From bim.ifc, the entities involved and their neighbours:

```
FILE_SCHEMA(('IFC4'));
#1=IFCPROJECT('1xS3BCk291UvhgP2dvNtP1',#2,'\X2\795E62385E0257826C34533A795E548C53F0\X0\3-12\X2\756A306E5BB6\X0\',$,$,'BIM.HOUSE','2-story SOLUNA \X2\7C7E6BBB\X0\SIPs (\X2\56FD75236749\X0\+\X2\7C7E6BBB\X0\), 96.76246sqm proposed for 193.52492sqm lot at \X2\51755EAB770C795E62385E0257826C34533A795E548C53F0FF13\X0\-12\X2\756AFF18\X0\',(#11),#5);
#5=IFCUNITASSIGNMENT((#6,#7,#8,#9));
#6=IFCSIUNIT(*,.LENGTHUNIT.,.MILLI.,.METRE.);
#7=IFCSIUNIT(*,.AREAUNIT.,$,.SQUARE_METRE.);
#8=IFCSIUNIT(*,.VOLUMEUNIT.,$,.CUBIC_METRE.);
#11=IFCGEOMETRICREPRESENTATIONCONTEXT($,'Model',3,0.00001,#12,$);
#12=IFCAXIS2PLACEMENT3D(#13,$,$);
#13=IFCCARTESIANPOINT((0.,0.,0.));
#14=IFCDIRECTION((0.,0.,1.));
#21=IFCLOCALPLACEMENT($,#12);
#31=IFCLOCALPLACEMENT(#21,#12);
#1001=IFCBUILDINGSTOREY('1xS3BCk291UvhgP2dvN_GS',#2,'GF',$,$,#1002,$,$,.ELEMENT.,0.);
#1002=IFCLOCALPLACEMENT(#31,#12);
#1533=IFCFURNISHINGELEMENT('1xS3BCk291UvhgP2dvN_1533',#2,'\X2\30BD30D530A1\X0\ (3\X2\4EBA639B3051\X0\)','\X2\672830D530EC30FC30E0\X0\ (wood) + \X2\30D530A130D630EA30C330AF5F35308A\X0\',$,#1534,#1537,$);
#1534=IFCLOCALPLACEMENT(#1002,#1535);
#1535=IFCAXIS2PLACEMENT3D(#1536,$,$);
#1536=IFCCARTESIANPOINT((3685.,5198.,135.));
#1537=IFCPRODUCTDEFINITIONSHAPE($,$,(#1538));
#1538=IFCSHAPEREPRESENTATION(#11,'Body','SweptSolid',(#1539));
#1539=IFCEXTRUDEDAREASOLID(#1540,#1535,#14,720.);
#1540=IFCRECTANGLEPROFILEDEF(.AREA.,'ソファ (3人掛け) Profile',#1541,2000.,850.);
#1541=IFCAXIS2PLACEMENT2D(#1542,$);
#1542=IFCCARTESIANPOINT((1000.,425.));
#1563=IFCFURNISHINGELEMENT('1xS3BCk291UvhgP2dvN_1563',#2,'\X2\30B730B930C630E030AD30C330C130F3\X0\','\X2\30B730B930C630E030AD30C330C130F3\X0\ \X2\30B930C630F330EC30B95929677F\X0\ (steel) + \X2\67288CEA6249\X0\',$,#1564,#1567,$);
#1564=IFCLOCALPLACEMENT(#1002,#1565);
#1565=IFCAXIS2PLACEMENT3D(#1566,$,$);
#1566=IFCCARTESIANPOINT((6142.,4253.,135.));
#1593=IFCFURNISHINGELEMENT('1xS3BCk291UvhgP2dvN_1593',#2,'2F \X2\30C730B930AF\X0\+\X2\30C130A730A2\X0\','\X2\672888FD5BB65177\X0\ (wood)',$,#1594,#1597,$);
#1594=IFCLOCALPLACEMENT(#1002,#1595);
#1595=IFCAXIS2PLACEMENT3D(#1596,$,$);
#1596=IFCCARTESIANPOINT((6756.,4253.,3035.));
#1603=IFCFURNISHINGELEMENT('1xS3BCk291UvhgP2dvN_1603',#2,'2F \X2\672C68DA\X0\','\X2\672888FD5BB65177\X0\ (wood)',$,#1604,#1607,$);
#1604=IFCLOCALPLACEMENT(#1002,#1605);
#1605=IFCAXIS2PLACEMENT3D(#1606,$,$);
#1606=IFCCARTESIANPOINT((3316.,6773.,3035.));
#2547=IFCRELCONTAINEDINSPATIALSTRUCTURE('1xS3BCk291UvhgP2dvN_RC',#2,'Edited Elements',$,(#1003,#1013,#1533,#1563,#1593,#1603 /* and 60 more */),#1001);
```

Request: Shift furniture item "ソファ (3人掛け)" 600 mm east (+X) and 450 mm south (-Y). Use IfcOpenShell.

```python
import ifcopenshell
import ifcopenshell.api.geometry
import ifcopenshell.util.placement
import ifcopenshell.util.unit

model = ifcopenshell.open("bim.ifc")
unit_scale = ifcopenshell.util.unit.calculate_unit_scale(model)

item = model.by_guid("1xS3BCk291UvhgP2dvN_1533")
matrix = ifcopenshell.util.placement.get_local_placement(item.ObjectPlacement)
matrix[0, 3] += 0.6 / unit_scale
matrix[1, 3] -= 0.45 / unit_scale
ifcopenshell.api.geometry.edit_object_placement(model, product=item, matrix=matrix, is_si=False)

print(ifcopenshell.util.placement.get_local_placement(item.ObjectPlacement).round(3) + 0.0)

model.write("bim_rev.ifc")
```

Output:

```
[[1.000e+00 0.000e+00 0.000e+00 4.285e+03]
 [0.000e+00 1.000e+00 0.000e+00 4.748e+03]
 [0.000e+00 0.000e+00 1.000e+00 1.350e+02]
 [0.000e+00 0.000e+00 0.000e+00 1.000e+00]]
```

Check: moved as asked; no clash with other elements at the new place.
